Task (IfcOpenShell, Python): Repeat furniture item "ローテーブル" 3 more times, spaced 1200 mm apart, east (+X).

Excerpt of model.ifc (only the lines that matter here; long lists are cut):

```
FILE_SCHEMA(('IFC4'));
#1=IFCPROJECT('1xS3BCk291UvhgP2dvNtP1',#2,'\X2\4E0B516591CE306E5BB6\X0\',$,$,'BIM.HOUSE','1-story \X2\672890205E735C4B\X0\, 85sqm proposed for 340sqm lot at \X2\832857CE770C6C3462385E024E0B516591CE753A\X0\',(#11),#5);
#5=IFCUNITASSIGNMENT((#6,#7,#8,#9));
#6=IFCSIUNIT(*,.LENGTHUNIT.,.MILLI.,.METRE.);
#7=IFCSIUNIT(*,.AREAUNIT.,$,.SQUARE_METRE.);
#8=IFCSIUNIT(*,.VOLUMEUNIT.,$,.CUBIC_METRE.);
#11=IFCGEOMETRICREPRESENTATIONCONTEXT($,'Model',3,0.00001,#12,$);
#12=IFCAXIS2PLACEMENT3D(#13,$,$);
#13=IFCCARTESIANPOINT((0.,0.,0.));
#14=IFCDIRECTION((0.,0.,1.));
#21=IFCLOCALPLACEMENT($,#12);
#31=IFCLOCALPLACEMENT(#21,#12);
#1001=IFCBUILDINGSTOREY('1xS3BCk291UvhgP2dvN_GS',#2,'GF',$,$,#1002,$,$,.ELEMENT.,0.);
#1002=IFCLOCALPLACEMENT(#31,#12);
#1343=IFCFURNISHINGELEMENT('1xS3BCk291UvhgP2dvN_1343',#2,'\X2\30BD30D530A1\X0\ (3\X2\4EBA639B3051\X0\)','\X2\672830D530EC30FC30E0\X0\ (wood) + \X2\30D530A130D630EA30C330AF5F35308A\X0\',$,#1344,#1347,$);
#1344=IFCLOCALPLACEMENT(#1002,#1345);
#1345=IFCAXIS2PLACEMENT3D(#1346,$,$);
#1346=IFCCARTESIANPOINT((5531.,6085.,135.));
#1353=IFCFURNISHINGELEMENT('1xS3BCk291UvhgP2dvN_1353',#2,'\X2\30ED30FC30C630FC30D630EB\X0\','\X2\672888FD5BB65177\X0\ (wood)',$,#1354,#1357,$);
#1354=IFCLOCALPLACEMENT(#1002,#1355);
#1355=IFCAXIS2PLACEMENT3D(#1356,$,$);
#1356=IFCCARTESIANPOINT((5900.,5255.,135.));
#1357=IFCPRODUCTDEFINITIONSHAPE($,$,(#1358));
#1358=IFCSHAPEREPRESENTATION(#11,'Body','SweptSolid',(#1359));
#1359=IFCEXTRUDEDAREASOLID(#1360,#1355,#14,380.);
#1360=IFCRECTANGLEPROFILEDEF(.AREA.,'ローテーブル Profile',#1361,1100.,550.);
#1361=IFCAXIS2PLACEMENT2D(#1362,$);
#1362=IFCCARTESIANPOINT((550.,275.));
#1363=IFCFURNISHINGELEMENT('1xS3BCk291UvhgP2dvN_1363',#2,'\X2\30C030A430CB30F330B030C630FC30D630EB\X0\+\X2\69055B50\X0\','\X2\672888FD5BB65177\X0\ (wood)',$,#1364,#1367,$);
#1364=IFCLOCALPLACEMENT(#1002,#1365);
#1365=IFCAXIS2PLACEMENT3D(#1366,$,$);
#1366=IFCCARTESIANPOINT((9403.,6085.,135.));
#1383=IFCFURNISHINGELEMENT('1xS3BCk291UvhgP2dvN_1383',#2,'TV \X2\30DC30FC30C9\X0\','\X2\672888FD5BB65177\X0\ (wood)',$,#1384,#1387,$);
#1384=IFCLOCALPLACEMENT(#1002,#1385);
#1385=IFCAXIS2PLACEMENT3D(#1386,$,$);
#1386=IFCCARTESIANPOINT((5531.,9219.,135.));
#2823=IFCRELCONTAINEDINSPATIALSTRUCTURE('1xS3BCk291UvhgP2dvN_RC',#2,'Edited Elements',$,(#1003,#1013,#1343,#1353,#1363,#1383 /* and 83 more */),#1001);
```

```python
import numpy as np
import ifcopenshell
import ifcopenshell.api.geometry
import ifcopenshell.api.root
import ifcopenshell.util.element
import ifcopenshell.util.placement
import ifcopenshell.util.unit

model = ifcopenshell.open("model.ifc")
unit_scale = ifcopenshell.util.unit.calculate_unit_scale(model)


def reuse_history(source, copy):
    """copy_class also copies each property set's owner history, people and application; keep the originals."""
    for rel in copy.IsDefinedBy:
        if rel.is_a("IfcRelDefinesByProperties") and (history := rel.RelatingPropertyDefinition.OwnerHistory):
            rel.RelatingPropertyDefinition.OwnerHistory = source.OwnerHistory
            ifcopenshell.util.element.remove_deep2(model, history)


source = model.by_guid("1xS3BCk291UvhgP2dvN_1353")
base = ifcopenshell.util.placement.get_local_placement(source.ObjectPlacement)
step = np.array([1.0, 0.0, 0.0]) * 1.2 / unit_scale

for i in range(1, 4):
    copy = ifcopenshell.api.root.copy_class(model, product=source)
    copy.Representation = ifcopenshell.util.element.copy_deep(
        model, source.Representation, exclude=["IfcGeometricRepresentationContext", "IfcRepresentationMap"]
    )
    reuse_history(source, copy)
    matrix = base.copy()
    matrix[:3, 3] += i * step
    print("added at", matrix[:3, 3].round(3) + 0.0)
    ifcopenshell.api.geometry.edit_object_placement(model, product=copy, matrix=matrix, is_si=False)

model.write("model_edited.ifc")
```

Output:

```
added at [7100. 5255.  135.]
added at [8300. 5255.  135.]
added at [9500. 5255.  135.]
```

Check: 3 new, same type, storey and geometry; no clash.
